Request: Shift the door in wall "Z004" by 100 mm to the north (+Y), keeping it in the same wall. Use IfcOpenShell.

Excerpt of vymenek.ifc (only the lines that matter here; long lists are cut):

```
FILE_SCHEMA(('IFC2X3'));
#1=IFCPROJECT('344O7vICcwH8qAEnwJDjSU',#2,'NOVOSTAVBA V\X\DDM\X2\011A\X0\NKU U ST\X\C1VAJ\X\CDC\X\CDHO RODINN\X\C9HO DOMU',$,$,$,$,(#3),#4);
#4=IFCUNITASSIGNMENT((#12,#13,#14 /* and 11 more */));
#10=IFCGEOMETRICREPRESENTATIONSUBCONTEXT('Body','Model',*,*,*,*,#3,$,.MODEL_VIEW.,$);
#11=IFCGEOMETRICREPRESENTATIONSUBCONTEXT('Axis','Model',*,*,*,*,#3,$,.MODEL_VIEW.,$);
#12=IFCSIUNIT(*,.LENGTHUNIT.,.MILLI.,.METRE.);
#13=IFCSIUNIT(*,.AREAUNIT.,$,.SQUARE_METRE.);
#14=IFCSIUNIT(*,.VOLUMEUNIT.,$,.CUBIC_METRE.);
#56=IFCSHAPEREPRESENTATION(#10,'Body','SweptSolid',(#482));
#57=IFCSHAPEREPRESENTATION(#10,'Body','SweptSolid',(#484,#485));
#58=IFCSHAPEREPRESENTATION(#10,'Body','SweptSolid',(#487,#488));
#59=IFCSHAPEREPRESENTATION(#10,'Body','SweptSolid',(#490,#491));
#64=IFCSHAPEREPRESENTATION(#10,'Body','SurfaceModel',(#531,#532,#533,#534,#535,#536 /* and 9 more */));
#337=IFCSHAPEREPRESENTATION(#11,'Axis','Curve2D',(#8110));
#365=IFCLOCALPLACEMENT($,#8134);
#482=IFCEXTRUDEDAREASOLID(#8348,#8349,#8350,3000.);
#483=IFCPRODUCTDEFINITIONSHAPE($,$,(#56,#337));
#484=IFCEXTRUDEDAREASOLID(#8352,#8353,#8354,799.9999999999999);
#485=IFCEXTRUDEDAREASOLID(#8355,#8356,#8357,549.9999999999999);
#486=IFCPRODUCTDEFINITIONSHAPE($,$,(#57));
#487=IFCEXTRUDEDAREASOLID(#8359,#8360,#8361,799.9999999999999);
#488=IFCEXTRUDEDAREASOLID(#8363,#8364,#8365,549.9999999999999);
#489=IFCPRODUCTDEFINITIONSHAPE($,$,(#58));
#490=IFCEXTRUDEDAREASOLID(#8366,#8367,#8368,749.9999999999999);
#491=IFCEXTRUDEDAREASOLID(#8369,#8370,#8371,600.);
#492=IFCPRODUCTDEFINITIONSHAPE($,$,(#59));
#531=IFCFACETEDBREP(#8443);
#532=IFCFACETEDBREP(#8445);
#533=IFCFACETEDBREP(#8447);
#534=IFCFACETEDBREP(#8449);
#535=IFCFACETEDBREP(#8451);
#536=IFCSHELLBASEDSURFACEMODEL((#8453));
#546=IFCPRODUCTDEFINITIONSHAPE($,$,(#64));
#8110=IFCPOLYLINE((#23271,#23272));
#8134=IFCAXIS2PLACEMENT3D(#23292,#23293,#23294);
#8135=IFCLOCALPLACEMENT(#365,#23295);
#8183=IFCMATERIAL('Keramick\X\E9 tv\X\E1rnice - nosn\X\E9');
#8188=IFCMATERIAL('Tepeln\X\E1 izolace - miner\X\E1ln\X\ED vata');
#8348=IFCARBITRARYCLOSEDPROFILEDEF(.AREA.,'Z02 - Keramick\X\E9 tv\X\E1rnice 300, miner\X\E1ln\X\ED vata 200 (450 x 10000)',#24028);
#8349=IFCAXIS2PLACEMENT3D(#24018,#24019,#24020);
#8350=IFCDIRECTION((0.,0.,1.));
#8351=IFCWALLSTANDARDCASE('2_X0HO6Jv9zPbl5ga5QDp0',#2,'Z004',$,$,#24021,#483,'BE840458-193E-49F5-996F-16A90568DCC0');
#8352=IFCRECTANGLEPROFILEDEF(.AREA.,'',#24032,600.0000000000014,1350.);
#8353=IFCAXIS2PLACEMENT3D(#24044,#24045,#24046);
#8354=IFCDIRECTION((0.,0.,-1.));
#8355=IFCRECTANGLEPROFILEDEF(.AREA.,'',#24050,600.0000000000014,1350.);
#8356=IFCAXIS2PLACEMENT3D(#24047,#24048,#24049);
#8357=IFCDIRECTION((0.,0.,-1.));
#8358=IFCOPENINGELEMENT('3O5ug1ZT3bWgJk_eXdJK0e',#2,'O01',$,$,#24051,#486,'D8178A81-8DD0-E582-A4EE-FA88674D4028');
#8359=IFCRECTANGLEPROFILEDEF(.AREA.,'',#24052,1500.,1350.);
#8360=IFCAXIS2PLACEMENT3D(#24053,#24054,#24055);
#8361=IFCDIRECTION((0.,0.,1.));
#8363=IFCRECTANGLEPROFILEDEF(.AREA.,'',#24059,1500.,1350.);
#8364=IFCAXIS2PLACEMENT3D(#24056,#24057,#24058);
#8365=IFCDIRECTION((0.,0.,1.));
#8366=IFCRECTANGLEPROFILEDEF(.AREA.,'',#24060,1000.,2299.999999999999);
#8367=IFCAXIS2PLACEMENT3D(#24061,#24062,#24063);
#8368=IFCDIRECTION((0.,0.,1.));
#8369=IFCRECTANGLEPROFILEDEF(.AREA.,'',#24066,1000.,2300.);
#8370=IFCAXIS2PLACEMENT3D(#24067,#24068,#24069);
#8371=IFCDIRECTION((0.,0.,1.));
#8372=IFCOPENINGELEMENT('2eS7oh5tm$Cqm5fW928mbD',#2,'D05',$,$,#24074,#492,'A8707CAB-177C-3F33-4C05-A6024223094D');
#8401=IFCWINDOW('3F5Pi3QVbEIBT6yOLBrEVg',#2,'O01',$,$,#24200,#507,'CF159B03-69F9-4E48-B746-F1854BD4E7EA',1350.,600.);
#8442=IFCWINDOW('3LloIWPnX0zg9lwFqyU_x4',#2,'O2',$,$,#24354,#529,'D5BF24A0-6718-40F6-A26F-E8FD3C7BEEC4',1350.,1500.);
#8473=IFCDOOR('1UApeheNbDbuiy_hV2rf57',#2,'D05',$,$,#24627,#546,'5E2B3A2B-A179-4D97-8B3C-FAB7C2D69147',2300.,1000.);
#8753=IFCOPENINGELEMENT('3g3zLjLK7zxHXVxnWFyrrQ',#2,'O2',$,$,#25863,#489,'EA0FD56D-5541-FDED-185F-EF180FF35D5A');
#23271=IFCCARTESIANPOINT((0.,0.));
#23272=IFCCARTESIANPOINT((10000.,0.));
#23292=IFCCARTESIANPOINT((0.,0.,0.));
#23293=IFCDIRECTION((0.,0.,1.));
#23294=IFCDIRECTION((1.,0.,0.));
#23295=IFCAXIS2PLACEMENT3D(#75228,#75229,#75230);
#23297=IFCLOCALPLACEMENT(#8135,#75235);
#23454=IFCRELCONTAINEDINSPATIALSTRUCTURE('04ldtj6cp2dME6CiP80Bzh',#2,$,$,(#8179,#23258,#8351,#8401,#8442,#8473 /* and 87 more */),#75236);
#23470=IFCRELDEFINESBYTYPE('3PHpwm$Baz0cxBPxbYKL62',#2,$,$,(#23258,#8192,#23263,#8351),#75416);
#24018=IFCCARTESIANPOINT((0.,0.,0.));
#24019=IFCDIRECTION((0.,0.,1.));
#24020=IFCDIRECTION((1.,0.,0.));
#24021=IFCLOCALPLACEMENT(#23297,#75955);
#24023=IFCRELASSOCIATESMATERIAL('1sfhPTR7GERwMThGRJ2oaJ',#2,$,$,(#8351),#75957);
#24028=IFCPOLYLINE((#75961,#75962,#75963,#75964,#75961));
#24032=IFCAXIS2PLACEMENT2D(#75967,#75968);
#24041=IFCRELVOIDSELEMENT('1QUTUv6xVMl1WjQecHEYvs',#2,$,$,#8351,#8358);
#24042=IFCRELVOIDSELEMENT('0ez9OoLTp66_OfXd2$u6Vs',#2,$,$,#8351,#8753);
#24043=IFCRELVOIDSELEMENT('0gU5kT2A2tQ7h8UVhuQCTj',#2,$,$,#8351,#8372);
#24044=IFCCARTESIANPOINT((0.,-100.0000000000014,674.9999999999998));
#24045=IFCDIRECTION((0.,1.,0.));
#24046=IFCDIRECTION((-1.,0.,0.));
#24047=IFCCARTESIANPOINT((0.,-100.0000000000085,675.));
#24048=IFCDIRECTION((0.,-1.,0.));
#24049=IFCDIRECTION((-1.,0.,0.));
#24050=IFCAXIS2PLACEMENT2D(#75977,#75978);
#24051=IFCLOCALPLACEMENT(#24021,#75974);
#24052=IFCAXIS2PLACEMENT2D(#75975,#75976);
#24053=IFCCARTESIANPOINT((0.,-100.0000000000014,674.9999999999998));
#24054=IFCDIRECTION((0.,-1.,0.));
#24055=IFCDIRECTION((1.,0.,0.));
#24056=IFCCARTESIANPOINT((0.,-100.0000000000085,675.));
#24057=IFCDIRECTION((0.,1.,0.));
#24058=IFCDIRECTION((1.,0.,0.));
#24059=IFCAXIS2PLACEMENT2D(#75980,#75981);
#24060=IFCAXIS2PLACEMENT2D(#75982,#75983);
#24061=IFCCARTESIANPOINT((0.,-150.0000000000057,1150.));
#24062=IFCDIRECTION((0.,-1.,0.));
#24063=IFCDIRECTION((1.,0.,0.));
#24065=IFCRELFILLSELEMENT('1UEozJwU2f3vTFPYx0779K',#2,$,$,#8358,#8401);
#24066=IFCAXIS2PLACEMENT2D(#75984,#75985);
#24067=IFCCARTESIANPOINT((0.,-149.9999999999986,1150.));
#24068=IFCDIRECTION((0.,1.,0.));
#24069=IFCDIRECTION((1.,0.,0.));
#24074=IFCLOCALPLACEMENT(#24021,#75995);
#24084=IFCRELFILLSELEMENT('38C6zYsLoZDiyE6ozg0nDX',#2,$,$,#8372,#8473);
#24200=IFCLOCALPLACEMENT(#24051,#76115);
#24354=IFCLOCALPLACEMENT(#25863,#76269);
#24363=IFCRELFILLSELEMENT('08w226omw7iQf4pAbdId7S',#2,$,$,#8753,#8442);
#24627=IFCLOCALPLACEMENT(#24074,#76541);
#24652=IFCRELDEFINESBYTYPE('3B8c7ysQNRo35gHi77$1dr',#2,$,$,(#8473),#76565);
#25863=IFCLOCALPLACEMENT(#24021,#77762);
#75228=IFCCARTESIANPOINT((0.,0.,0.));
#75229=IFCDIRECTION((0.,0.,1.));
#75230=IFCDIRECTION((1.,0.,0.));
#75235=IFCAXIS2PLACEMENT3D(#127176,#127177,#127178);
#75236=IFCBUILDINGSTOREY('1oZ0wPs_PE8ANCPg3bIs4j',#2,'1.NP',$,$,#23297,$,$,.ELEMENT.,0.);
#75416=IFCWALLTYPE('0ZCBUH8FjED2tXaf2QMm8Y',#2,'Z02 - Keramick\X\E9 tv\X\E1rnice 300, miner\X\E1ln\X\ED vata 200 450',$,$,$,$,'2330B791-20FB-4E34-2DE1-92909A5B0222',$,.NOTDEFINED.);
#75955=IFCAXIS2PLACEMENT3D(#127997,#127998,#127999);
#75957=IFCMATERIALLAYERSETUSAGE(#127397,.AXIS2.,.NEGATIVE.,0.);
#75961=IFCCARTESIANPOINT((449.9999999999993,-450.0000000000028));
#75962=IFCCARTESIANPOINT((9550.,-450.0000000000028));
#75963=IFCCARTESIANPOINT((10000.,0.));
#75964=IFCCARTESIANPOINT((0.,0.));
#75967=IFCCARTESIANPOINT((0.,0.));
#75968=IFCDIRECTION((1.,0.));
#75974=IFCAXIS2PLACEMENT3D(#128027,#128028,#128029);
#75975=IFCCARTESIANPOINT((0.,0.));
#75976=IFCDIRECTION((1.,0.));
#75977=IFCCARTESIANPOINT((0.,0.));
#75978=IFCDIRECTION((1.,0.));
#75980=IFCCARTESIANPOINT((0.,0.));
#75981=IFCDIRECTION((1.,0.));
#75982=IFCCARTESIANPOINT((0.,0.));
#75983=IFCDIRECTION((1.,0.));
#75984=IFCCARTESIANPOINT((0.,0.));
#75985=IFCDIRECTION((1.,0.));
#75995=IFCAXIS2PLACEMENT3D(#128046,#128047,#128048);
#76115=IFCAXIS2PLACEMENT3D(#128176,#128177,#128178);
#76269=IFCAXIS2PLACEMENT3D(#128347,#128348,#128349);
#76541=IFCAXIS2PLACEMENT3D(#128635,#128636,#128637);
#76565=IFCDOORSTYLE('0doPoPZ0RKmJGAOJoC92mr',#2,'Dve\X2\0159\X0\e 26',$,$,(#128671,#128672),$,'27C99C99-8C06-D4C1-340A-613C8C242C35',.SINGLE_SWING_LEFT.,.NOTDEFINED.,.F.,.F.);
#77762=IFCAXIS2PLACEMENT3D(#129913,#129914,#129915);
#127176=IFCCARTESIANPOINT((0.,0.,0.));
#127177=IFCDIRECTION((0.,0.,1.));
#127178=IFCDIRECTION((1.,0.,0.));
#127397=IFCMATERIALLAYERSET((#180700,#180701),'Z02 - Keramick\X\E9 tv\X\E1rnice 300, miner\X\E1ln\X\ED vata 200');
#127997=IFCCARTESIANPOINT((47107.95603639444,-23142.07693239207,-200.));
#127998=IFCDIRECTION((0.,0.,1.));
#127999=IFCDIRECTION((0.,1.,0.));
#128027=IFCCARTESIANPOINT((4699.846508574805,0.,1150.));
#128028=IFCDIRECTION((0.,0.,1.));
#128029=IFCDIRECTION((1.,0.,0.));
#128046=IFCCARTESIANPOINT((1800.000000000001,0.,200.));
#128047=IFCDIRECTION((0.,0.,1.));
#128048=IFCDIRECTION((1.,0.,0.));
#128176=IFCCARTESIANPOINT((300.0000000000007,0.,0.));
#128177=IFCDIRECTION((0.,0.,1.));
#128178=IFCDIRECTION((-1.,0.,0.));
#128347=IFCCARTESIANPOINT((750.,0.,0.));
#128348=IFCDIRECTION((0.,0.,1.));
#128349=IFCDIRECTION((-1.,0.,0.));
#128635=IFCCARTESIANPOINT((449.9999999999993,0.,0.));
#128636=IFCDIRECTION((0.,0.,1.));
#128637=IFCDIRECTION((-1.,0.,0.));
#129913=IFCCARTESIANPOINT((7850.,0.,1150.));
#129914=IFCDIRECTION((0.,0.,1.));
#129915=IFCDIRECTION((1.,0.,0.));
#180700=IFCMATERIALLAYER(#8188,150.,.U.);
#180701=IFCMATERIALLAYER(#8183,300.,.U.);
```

```python
import ifcopenshell
import ifcopenshell.api.geometry
import ifcopenshell.util.placement
import ifcopenshell.util.unit

model = ifcopenshell.open("vymenek.ifc")
unit_scale = ifcopenshell.util.unit.calculate_unit_scale(model)

door = model.by_guid("1UApeheNbDbuiy_hV2rf57")
opening = door.FillsVoids[0].RelatingOpeningElement
wall = opening.VoidsElements[0].RelatingBuildingElement

wall_matrix = ifcopenshell.util.placement.get_local_placement(wall.ObjectPlacement)
shift = wall_matrix[:3, 0] * 0.1 / unit_scale
before = ifcopenshell.util.placement.get_local_placement(door.ObjectPlacement)[:3, 3].copy()

# The door is placed relative to its opening, so it follows when the opening moves.
matrix = ifcopenshell.util.placement.get_local_placement(opening.ObjectPlacement)
matrix[:3, 3] += shift
ifcopenshell.api.geometry.edit_object_placement(
    model, product=opening, matrix=matrix, is_si=False, should_transform_children=True
)

after = ifcopenshell.util.placement.get_local_placement(door.ObjectPlacement)[:3, 3]
print("door moved by", (after - before).round(3) + 0.0)

model.write("vymenek_updated.ifc")
```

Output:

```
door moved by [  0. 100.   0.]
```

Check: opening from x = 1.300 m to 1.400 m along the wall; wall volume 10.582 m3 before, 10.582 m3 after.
